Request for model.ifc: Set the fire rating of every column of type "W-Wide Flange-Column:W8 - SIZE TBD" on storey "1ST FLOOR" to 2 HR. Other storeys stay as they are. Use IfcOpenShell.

First a look at what the model holds.

```python
import ifcopenshell
import ifcopenshell.util.element

model = ifcopenshell.open("model.ifc")
print(model.schema)
storey = next(s for s in model.by_type("IfcBuildingStorey") if s.Name == "1ST FLOOR")
columns = [e for e in ifcopenshell.util.element.get_decomposition(storey) if e.is_a("IfcColumn")]
seen = {}
for e in columns:
    element_type = ifcopenshell.util.element.get_type(e)
    key = (element_type.Name if element_type != e and element_type else None, ifcopenshell.util.element.get_pset(e, "Pset_ColumnCommon", "FireRating"))
    seen[key] = seen.get(key, 0) + 1
for (name, value), count in sorted(seen.items(), key=str):
    print(count, "x", name, "|", value)
```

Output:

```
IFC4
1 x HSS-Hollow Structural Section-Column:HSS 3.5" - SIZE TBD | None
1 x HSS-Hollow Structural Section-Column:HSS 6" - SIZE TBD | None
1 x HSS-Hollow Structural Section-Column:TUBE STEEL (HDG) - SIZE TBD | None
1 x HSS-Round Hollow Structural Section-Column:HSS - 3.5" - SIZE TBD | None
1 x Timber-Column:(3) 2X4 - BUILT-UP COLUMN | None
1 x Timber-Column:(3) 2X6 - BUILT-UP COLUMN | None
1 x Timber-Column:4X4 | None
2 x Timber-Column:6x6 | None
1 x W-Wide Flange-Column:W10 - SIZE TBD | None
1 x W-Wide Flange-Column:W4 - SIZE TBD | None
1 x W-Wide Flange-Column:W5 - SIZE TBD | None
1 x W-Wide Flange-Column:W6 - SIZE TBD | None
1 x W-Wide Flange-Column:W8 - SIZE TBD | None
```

```python
import ifcopenshell
import ifcopenshell.api.pset
import ifcopenshell.util.element

model = ifcopenshell.open("model.ifc")

storey = next(s for s in model.by_type("IfcBuildingStorey") if s.Name == "1ST FLOOR")
columns = [e for e in ifcopenshell.util.element.get_decomposition(storey) if e.is_a("IfcColumn")]

count = 0
for e in columns:
    element_type = ifcopenshell.util.element.get_type(e)
    if element_type in (None, e) or element_type.Name != "W-Wide Flange-Column:W8 - SIZE TBD":
        continue
    # add_pset returns the element's existing set when there is one.
    pset = ifcopenshell.api.pset.add_pset(model, product=e, name="Pset_ColumnCommon")
    ifcopenshell.api.pset.edit_pset(model, pset=pset, properties={"FireRating": "2 HR"})
    count += 1

print(count, "columns updated")

model.write("model_v2.ifc")
```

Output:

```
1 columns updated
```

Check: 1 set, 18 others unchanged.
